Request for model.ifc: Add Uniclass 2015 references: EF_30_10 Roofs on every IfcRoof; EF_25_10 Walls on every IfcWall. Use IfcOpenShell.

First a look at what the model holds.

```python
import ifcopenshell

model = ifcopenshell.open("model.ifc")
print(model.schema)
print("classifications:", [c.Name for c in model.by_type("IfcClassification")])
for ifc_class in ("IfcDoor", "IfcRoof", "IfcStair", "IfcWall", "IfcWindow"):
    print(ifc_class, len(model.by_type(ifc_class)))
```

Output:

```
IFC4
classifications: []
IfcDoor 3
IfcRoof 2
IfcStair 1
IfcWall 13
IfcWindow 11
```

```python
import ifcopenshell
import ifcopenshell.api.classification

model = ifcopenshell.open("model.ifc")

system = ifcopenshell.api.classification.add_classification(model, classification="Uniclass 2015")

codes = {
    "IfcRoof": ("EF_30_10", "Roofs"),
    "IfcWall": ("EF_25_10", "Walls"),
}
for ifc_class, (code, name) in codes.items():
    products = model.by_type(ifc_class)
    ifcopenshell.api.classification.add_reference(
        model, products=products, classification=system, identification=code, name=name
    )
    print(code, len(products))

model.write("model_updated.ifc")
```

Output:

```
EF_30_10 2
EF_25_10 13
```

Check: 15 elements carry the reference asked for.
